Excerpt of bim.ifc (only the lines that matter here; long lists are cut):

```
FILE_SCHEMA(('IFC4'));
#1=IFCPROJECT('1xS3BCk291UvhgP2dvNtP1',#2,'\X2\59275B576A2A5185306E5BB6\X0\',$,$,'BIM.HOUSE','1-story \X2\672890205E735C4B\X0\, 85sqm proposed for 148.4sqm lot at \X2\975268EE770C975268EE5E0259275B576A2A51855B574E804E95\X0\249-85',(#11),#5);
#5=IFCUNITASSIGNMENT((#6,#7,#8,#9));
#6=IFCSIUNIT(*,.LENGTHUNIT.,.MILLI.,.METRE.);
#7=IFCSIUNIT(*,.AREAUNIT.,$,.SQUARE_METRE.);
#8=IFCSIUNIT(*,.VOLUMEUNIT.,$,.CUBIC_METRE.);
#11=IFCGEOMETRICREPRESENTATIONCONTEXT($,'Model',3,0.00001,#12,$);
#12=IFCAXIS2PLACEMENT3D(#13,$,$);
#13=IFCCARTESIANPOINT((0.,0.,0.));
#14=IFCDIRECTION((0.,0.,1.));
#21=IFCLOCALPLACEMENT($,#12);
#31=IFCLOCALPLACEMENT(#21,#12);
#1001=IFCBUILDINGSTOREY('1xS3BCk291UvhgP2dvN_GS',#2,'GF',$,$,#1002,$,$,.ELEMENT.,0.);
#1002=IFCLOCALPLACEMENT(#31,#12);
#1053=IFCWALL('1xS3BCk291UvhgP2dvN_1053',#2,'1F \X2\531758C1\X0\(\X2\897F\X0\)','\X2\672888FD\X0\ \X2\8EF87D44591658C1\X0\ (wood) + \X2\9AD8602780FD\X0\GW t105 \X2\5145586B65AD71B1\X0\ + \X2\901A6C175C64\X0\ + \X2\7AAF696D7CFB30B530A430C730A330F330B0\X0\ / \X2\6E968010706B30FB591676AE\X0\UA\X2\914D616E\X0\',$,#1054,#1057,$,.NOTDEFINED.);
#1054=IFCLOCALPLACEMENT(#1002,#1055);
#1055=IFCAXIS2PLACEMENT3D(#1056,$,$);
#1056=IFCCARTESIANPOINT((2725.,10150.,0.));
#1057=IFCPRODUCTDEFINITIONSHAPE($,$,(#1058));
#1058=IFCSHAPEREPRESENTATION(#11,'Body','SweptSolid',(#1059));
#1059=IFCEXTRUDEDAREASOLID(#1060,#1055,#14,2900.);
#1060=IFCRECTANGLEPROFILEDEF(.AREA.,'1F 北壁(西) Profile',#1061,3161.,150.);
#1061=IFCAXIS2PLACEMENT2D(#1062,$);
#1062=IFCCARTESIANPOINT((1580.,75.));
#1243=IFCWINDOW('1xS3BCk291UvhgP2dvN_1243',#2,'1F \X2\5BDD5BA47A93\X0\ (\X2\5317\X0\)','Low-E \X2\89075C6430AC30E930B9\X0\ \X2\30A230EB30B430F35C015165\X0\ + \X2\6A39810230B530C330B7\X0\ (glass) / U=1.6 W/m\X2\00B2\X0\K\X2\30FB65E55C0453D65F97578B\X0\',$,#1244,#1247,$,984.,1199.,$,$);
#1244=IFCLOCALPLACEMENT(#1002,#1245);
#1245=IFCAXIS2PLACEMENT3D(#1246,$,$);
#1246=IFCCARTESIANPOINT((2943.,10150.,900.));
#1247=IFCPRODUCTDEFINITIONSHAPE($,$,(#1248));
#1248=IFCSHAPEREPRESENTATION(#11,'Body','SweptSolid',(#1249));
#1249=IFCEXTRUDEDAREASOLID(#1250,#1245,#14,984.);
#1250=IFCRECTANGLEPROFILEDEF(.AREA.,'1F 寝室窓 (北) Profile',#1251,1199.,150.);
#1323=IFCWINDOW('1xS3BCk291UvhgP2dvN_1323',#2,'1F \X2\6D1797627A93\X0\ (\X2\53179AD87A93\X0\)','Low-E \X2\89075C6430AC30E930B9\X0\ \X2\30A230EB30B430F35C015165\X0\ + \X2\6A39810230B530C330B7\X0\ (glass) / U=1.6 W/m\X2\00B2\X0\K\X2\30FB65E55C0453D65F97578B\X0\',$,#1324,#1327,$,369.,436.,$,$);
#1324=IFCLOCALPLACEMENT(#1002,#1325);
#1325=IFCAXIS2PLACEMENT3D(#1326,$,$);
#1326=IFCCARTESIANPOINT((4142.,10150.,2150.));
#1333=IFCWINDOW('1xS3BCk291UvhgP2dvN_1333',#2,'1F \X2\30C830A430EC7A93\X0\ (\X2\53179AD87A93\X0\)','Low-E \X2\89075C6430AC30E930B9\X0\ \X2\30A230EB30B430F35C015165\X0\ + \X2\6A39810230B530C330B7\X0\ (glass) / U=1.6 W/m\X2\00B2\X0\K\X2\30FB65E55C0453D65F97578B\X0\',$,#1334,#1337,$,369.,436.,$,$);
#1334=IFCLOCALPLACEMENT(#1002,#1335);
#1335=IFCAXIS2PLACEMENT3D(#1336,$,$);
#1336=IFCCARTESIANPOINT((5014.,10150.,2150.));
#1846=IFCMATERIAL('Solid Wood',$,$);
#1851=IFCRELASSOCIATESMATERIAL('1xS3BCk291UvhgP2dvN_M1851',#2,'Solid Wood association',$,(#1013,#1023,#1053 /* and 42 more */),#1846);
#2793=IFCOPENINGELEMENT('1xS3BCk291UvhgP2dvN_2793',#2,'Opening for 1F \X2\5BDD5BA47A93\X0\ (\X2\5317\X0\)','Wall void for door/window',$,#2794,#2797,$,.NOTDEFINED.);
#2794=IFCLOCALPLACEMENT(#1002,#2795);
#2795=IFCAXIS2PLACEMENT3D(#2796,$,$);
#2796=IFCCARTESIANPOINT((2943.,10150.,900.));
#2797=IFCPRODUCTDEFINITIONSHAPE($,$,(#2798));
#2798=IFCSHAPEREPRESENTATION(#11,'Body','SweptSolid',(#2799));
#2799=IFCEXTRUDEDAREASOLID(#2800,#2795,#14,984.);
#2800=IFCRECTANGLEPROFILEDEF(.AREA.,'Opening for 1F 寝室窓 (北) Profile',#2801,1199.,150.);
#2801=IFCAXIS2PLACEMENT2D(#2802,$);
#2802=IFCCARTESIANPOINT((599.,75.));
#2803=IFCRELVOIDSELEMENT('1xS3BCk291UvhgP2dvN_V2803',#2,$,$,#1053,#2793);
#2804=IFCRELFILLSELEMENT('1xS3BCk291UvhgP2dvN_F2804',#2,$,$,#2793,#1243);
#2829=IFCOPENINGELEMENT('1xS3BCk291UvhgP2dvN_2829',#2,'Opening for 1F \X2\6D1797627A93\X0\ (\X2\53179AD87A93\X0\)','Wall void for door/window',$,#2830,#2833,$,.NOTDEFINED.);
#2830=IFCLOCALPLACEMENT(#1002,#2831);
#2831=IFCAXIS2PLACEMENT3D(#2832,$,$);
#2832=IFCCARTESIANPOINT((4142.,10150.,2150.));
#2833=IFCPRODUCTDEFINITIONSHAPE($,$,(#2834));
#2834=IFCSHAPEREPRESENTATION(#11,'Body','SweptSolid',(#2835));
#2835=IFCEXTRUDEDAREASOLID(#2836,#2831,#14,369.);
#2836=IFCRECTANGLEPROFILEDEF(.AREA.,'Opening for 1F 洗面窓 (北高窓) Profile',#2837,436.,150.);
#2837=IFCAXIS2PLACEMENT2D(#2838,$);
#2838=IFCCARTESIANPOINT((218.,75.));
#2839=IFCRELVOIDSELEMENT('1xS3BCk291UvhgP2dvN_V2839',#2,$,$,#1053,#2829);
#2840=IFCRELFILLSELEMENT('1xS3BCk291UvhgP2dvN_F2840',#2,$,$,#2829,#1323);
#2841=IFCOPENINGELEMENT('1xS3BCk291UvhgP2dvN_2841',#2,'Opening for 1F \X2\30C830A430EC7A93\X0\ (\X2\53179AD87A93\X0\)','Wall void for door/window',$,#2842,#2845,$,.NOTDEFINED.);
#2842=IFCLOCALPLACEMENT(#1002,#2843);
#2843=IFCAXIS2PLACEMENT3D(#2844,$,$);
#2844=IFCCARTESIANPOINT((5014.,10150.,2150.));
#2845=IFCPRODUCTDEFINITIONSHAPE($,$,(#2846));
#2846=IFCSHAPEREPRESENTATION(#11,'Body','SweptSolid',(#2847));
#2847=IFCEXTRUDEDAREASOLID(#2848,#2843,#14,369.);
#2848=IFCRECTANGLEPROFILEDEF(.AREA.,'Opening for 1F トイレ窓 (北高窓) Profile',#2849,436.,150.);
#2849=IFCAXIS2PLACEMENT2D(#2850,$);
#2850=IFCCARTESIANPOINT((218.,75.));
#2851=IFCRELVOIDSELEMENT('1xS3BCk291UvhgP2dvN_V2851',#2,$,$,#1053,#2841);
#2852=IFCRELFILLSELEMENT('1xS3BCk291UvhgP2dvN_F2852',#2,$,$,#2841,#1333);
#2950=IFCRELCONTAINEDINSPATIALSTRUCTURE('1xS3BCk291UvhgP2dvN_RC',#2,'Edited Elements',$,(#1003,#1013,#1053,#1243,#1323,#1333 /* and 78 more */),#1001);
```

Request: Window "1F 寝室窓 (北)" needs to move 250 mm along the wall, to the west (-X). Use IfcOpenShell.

```python
import ifcopenshell
import ifcopenshell.api.geometry
import ifcopenshell.util.placement
import ifcopenshell.util.unit

model = ifcopenshell.open("bim.ifc")
unit_scale = ifcopenshell.util.unit.calculate_unit_scale(model)

window = model.by_guid("1xS3BCk291UvhgP2dvN_1243")
opening = window.FillsVoids[0].RelatingOpeningElement
wall = opening.VoidsElements[0].RelatingBuildingElement

wall_matrix = ifcopenshell.util.placement.get_local_placement(wall.ObjectPlacement)
shift = wall_matrix[:3, 0] * -0.25 / unit_scale
before = ifcopenshell.util.placement.get_local_placement(window.ObjectPlacement)[:3, 3].copy()

# The window is not placed relative to its opening, so move both.
for product in (opening, window):
    matrix = ifcopenshell.util.placement.get_local_placement(product.ObjectPlacement)
    matrix[:3, 3] += shift
    ifcopenshell.api.geometry.edit_object_placement(model, product=product, matrix=matrix, is_si=False)

after = ifcopenshell.util.placement.get_local_placement(window.ObjectPlacement)[:3, 3]
print("window moved by", (after - before).round(3) + 0.0)

model.write("bim_updated.ifc")
```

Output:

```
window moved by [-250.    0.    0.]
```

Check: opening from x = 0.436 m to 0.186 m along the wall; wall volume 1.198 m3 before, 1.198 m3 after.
